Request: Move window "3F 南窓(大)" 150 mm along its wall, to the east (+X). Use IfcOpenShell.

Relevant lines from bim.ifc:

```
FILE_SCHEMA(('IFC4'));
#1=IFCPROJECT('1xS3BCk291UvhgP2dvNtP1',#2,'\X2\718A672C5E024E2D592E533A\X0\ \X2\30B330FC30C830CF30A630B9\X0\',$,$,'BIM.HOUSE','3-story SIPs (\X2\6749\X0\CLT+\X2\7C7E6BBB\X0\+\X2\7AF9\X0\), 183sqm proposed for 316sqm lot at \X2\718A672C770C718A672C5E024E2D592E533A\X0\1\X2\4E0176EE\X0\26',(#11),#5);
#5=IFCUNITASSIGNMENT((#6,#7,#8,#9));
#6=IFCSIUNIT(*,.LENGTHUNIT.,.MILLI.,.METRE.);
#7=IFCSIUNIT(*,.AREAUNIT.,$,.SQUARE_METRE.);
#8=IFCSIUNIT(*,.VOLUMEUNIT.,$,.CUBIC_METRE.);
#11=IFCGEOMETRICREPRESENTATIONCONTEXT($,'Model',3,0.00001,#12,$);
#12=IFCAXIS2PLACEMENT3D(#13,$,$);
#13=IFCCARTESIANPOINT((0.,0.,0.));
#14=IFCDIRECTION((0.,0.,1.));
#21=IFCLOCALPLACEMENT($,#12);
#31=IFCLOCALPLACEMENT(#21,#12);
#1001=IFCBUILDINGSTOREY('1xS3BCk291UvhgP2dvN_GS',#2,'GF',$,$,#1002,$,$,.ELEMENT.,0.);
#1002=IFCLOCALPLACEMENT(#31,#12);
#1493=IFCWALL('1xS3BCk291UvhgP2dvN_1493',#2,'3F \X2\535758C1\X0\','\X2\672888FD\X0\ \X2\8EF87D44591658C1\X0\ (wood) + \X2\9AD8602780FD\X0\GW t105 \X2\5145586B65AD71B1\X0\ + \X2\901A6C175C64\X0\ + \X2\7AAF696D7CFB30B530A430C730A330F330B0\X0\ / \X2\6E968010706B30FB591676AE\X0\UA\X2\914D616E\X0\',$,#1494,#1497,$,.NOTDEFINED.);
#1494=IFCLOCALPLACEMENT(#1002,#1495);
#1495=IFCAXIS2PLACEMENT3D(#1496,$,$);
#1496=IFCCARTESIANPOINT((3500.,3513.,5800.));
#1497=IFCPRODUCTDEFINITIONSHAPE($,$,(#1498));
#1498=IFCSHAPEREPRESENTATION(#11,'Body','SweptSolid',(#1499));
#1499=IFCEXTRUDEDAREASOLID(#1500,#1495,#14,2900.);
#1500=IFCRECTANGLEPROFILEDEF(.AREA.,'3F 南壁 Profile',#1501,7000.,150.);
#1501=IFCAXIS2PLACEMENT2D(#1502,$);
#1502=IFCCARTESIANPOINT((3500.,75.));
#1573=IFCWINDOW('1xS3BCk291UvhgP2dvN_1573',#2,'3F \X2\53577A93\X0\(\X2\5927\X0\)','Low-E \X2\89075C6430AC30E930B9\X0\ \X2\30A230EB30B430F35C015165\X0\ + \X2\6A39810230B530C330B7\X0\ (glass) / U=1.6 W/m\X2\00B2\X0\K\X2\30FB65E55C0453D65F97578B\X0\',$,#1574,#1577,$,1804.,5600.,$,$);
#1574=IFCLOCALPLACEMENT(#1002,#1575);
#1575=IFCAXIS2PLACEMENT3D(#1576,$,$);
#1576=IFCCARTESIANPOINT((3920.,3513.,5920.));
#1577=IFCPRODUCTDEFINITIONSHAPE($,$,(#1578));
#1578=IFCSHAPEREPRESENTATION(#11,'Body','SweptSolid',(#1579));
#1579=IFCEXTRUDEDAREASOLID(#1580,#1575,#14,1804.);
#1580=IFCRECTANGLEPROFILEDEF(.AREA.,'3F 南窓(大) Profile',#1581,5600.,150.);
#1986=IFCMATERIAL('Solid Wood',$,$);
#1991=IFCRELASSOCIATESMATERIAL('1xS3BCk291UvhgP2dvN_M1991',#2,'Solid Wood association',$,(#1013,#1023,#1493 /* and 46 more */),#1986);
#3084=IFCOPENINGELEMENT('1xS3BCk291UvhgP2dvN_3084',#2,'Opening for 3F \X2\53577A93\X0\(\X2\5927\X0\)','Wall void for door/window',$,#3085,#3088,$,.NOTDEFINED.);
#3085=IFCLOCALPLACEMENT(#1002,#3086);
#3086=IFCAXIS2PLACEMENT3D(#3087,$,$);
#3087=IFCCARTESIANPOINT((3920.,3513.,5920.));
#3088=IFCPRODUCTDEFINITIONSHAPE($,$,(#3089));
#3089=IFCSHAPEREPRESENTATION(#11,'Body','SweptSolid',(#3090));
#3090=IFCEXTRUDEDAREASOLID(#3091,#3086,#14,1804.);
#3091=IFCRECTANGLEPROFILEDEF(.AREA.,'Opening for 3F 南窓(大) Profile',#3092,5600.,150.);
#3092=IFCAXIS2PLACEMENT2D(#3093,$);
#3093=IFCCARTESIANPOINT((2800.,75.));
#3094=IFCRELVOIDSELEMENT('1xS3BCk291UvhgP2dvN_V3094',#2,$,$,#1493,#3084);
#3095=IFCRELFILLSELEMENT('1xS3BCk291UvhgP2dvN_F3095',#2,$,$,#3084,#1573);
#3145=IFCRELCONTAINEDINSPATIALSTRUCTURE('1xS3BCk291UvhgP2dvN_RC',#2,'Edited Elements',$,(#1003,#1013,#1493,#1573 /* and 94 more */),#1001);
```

```python
import ifcopenshell
import ifcopenshell.api.geometry
import ifcopenshell.util.placement

model = ifcopenshell.open("bim.ifc")

window = model.by_guid("1xS3BCk291UvhgP2dvN_1573")
opening = window.FillsVoids[0].RelatingOpeningElement
wall = opening.VoidsElements[0].RelatingBuildingElement

wall_matrix = ifcopenshell.util.placement.get_local_placement(wall.ObjectPlacement)
shift = wall_matrix[:3, 0] * 150.0
before = ifcopenshell.util.placement.get_local_placement(window.ObjectPlacement)[:3, 3].copy()

# The window is not placed relative to its opening, so move both.
for product in (opening, window):
    matrix = ifcopenshell.util.placement.get_local_placement(product.ObjectPlacement)
    matrix[:3, 3] += shift
    ifcopenshell.api.geometry.edit_object_placement(model, product=product, matrix=matrix, is_si=False)

after = ifcopenshell.util.placement.get_local_placement(window.ObjectPlacement)[:3, 3]
print("window moved by", (after - before).round(3) + 0.0)

model.write("bim_updated.ifc")
```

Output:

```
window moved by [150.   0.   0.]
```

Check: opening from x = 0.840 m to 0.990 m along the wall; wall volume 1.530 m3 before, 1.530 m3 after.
